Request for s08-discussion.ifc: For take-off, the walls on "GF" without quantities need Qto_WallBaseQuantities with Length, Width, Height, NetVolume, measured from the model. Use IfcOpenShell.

First a look at what the model holds.

```python
import ifcopenshell
import ifcopenshell.util.element
import ifcopenshell.util.unit

model = ifcopenshell.open("s08-discussion.ifc")
print(model.schema)
for unit_type in ("LENGTHUNIT", "AREAUNIT", "VOLUMEUNIT"):
    print(unit_type, ifcopenshell.util.unit.calculate_unit_scale(model, unit_type))
storey = next(s for s in model.by_type("IfcBuildingStorey") if s.Name == "GF")
walls = [e for e in ifcopenshell.util.element.get_decomposition(storey) if e.is_a("IfcWall")]
for e in sorted(walls, key=lambda e: e.id()):
    print(e.id(), e.is_a(), e.Name, list(ifcopenshell.util.element.get_psets(e, qtos_only=True)), sep=" | ")
```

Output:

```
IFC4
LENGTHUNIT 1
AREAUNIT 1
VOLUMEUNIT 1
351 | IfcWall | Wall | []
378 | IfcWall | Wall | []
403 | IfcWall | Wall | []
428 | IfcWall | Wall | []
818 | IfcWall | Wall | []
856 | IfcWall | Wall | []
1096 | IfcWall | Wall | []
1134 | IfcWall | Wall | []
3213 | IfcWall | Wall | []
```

```python
import ifcopenshell
import ifcopenshell.api.pset
import ifcopenshell.geom
import ifcopenshell.util.element
import ifcopenshell.util.shape
import ifcopenshell.util.unit

model = ifcopenshell.open("s08-discussion.ifc")
unit_scale = ifcopenshell.util.unit.calculate_unit_scale(model)
volume_scale = ifcopenshell.util.unit.calculate_unit_scale(model, "VOLUMEUNIT")
settings = ifcopenshell.geom.settings()

storey = next(s for s in model.by_type("IfcBuildingStorey") if s.Name == "GF")
walls = [e for e in ifcopenshell.util.element.get_decomposition(storey) if e.is_a("IfcWall")]

for e in sorted(walls, key=lambda e: e.id()):
    if ifcopenshell.util.element.get_psets(e, qtos_only=True, should_inherit=False):
        continue
    # Geometry comes back in metres, in the element's own axes.
    shape = ifcopenshell.geom.create_shape(settings, e)
    values = {
        "Length": ifcopenshell.util.shape.get_x(shape.geometry) / unit_scale,
        "Width": ifcopenshell.util.shape.get_y(shape.geometry) / unit_scale,
        "Height": ifcopenshell.util.shape.get_z(shape.geometry) / unit_scale,
        "NetVolume": ifcopenshell.util.shape.get_volume(shape.geometry) / volume_scale,
    }
    qto = ifcopenshell.api.pset.add_qto(model, product=e, name="Qto_WallBaseQuantities")
    ifcopenshell.api.pset.edit_qto(model, qto=qto, properties=values)
    print(e.id(), {k: round(v, 3) for k, v in values.items()})

model.write("s08-discussion_v2.ifc")
```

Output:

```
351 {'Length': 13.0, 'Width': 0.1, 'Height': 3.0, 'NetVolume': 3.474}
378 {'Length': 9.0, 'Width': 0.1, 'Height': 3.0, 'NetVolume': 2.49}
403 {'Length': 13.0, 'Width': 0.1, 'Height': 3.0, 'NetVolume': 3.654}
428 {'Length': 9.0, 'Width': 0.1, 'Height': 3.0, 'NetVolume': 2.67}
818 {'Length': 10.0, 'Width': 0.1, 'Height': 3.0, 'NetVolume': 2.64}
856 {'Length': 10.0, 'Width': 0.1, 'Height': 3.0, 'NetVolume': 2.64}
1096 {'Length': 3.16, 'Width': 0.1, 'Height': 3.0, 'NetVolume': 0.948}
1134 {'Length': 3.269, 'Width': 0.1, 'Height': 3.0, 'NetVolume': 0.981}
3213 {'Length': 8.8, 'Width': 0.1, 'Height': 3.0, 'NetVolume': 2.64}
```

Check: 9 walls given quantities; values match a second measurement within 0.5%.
